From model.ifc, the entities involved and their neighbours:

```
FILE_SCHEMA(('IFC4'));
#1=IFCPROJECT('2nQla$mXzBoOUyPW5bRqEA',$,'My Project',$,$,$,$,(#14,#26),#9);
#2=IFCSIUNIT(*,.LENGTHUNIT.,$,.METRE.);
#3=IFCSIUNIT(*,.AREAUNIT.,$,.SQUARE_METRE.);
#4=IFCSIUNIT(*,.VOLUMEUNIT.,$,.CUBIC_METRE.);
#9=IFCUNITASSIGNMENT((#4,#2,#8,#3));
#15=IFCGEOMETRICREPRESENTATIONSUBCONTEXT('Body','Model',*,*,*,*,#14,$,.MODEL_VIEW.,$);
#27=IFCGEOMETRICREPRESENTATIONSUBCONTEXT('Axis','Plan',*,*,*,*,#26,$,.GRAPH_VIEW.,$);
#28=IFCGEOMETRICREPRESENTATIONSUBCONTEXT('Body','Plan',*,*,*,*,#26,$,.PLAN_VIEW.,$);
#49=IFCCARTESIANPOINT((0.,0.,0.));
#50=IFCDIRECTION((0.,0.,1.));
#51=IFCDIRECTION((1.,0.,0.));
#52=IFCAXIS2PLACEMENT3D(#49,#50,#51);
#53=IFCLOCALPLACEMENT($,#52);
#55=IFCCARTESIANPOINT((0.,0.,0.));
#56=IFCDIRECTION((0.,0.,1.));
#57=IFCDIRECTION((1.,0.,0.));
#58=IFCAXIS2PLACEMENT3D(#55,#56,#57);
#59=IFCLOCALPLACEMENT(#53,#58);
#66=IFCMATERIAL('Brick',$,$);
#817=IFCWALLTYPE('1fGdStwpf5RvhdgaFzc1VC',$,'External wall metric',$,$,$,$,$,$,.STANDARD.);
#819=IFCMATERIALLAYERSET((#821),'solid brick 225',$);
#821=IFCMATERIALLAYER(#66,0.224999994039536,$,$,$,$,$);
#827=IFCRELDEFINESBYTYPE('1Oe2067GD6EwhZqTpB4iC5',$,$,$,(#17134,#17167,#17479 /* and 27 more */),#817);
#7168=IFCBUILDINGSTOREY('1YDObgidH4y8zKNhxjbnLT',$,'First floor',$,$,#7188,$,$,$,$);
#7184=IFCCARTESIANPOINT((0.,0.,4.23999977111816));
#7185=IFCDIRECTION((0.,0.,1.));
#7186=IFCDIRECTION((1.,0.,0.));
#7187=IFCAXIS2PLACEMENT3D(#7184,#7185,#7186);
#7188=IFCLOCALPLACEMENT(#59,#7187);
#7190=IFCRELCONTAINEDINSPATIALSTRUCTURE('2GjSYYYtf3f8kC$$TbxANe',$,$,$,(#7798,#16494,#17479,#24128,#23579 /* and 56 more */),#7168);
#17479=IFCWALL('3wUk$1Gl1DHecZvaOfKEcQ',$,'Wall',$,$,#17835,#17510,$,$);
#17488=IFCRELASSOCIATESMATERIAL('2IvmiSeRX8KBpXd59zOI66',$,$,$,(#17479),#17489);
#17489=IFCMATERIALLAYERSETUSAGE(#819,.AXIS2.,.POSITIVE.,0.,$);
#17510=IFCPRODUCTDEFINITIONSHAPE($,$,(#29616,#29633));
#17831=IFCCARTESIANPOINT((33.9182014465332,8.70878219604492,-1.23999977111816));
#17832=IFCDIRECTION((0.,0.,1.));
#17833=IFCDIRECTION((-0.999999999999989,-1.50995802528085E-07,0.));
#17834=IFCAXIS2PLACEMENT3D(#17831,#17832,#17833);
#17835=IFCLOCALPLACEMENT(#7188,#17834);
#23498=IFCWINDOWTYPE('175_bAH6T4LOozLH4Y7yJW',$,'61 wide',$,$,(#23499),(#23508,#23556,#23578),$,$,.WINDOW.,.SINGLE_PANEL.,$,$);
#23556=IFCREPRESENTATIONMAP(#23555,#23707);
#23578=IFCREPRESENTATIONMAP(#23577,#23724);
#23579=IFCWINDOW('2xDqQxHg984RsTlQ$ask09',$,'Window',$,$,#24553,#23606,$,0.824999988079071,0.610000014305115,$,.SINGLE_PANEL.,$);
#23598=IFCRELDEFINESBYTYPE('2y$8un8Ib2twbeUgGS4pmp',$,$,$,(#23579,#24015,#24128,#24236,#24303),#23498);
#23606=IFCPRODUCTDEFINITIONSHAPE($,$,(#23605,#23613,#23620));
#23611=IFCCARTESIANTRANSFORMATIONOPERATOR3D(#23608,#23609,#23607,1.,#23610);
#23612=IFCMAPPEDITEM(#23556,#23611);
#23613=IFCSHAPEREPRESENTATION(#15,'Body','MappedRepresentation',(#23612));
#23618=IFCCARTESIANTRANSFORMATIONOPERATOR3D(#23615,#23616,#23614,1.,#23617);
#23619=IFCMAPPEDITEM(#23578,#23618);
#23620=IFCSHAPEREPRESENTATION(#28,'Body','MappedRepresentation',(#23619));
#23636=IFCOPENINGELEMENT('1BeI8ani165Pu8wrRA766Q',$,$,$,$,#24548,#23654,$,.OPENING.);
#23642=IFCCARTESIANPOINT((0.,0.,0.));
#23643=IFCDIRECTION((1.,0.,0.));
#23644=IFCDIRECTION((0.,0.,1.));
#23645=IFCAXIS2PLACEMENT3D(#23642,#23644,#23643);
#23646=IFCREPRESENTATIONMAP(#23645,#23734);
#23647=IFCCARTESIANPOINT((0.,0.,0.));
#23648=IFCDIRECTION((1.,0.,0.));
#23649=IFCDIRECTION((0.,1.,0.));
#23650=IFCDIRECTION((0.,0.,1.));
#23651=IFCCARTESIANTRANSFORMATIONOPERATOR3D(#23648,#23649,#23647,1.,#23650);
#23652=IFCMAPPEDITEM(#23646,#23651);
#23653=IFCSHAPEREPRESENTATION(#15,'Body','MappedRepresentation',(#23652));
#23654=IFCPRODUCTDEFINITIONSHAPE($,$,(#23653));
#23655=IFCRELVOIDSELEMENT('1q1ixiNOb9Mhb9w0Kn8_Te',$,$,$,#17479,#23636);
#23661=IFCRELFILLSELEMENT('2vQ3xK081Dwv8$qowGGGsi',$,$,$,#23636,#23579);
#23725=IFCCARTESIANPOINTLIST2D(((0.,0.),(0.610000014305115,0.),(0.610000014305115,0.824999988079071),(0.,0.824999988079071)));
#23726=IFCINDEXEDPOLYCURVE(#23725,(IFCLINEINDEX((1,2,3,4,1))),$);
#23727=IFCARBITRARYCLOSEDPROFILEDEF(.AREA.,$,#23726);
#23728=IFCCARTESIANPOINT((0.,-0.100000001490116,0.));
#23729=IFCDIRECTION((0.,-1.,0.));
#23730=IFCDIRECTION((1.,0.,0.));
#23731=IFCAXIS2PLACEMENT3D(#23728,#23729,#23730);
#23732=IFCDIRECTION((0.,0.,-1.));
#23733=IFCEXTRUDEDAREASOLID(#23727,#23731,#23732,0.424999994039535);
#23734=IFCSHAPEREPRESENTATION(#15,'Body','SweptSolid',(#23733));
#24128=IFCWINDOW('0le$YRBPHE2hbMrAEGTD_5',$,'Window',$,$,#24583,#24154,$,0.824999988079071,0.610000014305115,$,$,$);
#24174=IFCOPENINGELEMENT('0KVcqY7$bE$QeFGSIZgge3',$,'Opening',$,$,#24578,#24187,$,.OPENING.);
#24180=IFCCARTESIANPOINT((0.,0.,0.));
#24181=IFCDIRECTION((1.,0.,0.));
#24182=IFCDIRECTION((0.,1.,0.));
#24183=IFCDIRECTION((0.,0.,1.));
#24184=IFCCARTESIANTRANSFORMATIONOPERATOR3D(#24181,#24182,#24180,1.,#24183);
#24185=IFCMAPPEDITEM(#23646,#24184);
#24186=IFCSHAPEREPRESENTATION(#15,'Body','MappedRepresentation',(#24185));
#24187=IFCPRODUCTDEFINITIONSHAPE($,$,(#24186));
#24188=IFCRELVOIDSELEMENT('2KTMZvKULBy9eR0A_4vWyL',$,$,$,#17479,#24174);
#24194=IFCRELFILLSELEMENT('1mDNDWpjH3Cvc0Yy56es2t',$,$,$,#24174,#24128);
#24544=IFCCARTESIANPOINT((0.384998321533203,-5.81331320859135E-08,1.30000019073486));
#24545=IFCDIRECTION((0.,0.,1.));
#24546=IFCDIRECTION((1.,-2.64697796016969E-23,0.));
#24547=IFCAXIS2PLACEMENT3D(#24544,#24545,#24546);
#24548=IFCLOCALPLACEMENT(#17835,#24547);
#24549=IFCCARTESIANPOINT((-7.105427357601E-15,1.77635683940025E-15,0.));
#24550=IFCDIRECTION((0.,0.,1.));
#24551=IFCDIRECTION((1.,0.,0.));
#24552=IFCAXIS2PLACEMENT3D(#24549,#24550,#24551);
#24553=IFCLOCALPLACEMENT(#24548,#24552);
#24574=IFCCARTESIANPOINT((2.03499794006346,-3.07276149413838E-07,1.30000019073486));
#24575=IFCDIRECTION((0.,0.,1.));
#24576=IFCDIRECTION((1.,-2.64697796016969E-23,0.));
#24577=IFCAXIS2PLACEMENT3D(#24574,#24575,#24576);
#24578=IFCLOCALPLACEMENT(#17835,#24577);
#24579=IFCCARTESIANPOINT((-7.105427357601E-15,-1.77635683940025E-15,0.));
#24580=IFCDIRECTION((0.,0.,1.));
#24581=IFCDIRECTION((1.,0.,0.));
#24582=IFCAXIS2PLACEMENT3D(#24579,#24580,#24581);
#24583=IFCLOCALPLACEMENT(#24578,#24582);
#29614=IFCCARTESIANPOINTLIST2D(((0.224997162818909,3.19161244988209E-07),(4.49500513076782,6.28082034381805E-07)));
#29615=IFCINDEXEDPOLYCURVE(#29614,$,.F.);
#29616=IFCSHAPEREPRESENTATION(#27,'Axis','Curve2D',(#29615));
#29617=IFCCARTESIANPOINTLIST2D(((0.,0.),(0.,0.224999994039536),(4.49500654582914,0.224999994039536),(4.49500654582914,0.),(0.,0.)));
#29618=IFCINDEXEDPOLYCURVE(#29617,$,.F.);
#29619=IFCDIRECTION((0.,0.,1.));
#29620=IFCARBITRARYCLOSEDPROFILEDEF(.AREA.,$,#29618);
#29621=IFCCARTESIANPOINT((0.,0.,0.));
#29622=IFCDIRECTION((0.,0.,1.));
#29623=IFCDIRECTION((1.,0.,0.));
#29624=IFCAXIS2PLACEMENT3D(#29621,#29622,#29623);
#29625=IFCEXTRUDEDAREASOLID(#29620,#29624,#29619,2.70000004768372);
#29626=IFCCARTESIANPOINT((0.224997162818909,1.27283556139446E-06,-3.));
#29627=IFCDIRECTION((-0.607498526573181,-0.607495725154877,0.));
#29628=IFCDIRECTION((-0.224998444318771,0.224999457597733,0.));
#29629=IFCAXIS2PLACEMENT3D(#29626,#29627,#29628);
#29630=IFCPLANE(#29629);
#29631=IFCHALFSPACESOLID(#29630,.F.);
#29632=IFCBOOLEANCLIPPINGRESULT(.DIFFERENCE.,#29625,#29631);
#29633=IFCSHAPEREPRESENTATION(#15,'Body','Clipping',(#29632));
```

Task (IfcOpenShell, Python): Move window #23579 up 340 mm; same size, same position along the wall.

```python
import numpy as np
import ifcopenshell
import ifcopenshell.api.geometry
import ifcopenshell.util.placement
import ifcopenshell.util.unit

model = ifcopenshell.open("model.ifc")
unit_scale = ifcopenshell.util.unit.calculate_unit_scale(model)

window = model.by_guid("2xDqQxHg984RsTlQ$ask09")
opening = window.FillsVoids[0].RelatingOpeningElement
dz = 0.34 / unit_scale

shift = np.array([0.0, 0.0, dz])
# The window is placed relative to its opening, so it follows when the opening moves.
matrix = ifcopenshell.util.placement.get_local_placement(opening.ObjectPlacement)
matrix[:3, 3] += shift
ifcopenshell.api.geometry.edit_object_placement(
    model, product=opening, matrix=matrix, is_si=False, should_transform_children=True
)

print(f"moved by {dz * unit_scale:+.3f} m")

model.write("model_updated.ifc")
```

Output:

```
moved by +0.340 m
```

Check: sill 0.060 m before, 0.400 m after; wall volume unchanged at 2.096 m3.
